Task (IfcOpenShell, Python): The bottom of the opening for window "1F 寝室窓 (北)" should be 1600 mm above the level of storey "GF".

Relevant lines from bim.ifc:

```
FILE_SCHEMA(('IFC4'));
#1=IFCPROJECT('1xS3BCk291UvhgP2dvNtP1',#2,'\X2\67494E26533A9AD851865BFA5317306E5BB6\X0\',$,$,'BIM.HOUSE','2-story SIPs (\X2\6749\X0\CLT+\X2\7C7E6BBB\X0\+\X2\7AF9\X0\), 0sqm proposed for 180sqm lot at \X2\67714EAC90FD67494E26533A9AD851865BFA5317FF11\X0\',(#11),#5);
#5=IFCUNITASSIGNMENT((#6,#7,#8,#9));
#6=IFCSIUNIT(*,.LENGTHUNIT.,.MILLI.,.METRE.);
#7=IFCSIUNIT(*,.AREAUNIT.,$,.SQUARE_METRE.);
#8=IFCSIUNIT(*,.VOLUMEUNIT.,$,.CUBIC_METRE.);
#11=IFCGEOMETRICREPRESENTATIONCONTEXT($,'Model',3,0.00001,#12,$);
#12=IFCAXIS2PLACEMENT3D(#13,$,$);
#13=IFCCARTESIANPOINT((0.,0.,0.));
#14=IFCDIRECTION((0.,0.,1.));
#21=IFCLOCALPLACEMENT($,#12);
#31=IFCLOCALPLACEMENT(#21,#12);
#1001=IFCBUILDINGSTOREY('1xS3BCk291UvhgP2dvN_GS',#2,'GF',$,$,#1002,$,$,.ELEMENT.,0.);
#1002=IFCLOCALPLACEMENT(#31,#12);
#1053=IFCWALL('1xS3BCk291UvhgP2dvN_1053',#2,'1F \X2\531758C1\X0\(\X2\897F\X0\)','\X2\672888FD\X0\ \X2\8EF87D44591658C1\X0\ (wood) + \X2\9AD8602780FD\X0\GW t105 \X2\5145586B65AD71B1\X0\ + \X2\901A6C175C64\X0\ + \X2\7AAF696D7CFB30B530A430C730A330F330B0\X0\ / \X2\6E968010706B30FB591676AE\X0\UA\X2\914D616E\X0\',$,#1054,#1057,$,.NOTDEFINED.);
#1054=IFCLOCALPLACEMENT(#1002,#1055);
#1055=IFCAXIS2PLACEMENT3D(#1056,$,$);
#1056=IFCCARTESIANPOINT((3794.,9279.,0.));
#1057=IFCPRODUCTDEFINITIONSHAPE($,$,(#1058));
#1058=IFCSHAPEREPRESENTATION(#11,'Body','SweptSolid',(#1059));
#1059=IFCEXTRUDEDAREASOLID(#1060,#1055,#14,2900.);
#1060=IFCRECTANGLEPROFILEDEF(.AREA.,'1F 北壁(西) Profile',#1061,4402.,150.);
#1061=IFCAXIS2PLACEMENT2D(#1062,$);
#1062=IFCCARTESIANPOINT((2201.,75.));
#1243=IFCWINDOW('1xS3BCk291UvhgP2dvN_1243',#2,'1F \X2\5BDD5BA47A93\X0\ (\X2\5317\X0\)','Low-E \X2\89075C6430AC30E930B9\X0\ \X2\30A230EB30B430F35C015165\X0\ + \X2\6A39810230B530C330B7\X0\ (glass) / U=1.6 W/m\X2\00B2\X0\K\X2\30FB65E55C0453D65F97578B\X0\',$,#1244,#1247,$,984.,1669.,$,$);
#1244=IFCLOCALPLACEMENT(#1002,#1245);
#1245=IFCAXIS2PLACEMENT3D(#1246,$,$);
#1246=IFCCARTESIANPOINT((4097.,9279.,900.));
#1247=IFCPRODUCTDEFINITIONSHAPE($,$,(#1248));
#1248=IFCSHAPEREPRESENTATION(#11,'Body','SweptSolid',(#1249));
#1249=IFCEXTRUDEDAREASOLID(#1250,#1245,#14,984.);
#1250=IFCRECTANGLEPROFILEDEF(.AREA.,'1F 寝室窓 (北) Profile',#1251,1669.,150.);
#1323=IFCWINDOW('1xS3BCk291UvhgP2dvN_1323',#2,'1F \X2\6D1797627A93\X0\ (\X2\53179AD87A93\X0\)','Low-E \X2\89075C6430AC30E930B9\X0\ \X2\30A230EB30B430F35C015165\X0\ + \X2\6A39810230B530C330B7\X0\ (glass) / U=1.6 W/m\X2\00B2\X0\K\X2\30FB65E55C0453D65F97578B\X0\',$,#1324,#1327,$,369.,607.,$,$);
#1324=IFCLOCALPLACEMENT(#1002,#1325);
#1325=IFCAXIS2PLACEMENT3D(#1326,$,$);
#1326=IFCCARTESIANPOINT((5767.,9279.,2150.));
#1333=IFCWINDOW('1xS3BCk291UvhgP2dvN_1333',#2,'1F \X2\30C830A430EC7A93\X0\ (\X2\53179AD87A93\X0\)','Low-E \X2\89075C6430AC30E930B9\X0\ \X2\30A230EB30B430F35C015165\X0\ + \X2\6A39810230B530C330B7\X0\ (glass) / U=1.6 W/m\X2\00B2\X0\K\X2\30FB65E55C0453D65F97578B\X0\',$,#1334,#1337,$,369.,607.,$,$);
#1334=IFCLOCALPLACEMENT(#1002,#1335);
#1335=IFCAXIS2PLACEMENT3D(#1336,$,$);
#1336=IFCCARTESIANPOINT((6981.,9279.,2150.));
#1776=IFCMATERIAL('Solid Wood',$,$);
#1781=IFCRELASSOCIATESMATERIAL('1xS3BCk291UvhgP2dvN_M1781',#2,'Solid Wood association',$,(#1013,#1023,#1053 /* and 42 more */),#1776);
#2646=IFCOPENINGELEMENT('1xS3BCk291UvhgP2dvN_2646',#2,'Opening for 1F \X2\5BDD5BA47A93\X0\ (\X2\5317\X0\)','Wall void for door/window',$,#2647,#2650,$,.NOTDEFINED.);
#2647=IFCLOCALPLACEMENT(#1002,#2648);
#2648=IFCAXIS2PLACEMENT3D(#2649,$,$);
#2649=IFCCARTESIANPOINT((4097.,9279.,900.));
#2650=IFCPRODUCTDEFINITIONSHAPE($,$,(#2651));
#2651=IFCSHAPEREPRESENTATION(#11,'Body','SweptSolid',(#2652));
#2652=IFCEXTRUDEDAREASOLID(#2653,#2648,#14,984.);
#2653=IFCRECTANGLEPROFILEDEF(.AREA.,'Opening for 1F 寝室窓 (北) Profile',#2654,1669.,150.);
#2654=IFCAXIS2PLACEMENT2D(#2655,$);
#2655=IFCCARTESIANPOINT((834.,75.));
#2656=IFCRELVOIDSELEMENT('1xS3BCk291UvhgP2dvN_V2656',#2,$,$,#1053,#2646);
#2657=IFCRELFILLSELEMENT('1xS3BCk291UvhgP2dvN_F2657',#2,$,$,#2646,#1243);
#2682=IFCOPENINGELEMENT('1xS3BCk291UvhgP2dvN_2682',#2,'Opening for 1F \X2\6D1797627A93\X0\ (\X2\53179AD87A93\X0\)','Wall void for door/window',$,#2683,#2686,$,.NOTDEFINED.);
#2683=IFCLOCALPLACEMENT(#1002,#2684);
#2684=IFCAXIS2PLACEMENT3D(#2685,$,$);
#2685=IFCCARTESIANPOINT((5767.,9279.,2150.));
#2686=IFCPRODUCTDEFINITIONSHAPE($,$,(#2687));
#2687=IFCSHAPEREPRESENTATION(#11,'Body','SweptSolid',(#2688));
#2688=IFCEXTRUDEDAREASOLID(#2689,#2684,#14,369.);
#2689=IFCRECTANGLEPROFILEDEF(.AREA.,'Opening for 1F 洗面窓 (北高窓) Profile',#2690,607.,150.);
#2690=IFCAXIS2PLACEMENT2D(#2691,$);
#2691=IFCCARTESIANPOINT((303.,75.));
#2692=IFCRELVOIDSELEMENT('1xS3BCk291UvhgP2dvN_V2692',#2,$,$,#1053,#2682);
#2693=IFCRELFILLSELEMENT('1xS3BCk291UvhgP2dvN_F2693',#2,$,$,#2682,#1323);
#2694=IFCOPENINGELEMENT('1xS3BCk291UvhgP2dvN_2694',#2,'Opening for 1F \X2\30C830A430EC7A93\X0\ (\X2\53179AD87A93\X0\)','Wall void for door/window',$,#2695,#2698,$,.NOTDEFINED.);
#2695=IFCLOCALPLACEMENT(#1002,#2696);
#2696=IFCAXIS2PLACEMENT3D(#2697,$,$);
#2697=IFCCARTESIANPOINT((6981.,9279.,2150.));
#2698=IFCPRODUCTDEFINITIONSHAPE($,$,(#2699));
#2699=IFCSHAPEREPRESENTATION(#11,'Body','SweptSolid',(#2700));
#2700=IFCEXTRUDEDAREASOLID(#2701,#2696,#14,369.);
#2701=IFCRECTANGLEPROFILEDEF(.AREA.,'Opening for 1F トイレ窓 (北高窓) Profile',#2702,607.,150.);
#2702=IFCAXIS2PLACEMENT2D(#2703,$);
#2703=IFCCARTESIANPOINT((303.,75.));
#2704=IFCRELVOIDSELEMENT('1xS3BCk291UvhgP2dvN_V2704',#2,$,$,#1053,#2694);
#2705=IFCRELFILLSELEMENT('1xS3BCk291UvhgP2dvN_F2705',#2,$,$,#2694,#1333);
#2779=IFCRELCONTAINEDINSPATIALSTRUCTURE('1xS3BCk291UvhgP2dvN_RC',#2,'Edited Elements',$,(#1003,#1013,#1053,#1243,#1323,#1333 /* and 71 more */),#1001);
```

```python
import numpy as np
import ifcopenshell
import ifcopenshell.api.geometry
import ifcopenshell.geom
import ifcopenshell.util.element
import ifcopenshell.util.placement
import ifcopenshell.util.shape
import ifcopenshell.util.unit

model = ifcopenshell.open("bim.ifc")
unit_scale = ifcopenshell.util.unit.calculate_unit_scale(model)

window = model.by_id(1243)
opening = window.FillsVoids[0].RelatingOpeningElement
storey = ifcopenshell.util.element.get_container(window, ifc_class="IfcBuildingStorey")
level = ifcopenshell.util.placement.get_local_placement(storey.ObjectPlacement)[2, 3]

# The opening's origin need not be at the sill, so measure its lowest point.
shape = ifcopenshell.geom.create_shape(ifcopenshell.geom.settings(), opening)
bottom = ifcopenshell.util.shape.get_shape_bottom_elevation(shape, shape.geometry) / unit_scale
dz = level + 1.6 / unit_scale - bottom

shift = np.array([0.0, 0.0, dz])
# The window is not placed relative to its opening, so move both.
for product in (opening, window):
    matrix = ifcopenshell.util.placement.get_local_placement(product.ObjectPlacement)
    matrix[:3, 3] += shift
    ifcopenshell.api.geometry.edit_object_placement(model, product=product, matrix=matrix, is_si=False)

print(f"moved by {dz * unit_scale:+.3f} m")

model.write("bim_edited.ifc")
```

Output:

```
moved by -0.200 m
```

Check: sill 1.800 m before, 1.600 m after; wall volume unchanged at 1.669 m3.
